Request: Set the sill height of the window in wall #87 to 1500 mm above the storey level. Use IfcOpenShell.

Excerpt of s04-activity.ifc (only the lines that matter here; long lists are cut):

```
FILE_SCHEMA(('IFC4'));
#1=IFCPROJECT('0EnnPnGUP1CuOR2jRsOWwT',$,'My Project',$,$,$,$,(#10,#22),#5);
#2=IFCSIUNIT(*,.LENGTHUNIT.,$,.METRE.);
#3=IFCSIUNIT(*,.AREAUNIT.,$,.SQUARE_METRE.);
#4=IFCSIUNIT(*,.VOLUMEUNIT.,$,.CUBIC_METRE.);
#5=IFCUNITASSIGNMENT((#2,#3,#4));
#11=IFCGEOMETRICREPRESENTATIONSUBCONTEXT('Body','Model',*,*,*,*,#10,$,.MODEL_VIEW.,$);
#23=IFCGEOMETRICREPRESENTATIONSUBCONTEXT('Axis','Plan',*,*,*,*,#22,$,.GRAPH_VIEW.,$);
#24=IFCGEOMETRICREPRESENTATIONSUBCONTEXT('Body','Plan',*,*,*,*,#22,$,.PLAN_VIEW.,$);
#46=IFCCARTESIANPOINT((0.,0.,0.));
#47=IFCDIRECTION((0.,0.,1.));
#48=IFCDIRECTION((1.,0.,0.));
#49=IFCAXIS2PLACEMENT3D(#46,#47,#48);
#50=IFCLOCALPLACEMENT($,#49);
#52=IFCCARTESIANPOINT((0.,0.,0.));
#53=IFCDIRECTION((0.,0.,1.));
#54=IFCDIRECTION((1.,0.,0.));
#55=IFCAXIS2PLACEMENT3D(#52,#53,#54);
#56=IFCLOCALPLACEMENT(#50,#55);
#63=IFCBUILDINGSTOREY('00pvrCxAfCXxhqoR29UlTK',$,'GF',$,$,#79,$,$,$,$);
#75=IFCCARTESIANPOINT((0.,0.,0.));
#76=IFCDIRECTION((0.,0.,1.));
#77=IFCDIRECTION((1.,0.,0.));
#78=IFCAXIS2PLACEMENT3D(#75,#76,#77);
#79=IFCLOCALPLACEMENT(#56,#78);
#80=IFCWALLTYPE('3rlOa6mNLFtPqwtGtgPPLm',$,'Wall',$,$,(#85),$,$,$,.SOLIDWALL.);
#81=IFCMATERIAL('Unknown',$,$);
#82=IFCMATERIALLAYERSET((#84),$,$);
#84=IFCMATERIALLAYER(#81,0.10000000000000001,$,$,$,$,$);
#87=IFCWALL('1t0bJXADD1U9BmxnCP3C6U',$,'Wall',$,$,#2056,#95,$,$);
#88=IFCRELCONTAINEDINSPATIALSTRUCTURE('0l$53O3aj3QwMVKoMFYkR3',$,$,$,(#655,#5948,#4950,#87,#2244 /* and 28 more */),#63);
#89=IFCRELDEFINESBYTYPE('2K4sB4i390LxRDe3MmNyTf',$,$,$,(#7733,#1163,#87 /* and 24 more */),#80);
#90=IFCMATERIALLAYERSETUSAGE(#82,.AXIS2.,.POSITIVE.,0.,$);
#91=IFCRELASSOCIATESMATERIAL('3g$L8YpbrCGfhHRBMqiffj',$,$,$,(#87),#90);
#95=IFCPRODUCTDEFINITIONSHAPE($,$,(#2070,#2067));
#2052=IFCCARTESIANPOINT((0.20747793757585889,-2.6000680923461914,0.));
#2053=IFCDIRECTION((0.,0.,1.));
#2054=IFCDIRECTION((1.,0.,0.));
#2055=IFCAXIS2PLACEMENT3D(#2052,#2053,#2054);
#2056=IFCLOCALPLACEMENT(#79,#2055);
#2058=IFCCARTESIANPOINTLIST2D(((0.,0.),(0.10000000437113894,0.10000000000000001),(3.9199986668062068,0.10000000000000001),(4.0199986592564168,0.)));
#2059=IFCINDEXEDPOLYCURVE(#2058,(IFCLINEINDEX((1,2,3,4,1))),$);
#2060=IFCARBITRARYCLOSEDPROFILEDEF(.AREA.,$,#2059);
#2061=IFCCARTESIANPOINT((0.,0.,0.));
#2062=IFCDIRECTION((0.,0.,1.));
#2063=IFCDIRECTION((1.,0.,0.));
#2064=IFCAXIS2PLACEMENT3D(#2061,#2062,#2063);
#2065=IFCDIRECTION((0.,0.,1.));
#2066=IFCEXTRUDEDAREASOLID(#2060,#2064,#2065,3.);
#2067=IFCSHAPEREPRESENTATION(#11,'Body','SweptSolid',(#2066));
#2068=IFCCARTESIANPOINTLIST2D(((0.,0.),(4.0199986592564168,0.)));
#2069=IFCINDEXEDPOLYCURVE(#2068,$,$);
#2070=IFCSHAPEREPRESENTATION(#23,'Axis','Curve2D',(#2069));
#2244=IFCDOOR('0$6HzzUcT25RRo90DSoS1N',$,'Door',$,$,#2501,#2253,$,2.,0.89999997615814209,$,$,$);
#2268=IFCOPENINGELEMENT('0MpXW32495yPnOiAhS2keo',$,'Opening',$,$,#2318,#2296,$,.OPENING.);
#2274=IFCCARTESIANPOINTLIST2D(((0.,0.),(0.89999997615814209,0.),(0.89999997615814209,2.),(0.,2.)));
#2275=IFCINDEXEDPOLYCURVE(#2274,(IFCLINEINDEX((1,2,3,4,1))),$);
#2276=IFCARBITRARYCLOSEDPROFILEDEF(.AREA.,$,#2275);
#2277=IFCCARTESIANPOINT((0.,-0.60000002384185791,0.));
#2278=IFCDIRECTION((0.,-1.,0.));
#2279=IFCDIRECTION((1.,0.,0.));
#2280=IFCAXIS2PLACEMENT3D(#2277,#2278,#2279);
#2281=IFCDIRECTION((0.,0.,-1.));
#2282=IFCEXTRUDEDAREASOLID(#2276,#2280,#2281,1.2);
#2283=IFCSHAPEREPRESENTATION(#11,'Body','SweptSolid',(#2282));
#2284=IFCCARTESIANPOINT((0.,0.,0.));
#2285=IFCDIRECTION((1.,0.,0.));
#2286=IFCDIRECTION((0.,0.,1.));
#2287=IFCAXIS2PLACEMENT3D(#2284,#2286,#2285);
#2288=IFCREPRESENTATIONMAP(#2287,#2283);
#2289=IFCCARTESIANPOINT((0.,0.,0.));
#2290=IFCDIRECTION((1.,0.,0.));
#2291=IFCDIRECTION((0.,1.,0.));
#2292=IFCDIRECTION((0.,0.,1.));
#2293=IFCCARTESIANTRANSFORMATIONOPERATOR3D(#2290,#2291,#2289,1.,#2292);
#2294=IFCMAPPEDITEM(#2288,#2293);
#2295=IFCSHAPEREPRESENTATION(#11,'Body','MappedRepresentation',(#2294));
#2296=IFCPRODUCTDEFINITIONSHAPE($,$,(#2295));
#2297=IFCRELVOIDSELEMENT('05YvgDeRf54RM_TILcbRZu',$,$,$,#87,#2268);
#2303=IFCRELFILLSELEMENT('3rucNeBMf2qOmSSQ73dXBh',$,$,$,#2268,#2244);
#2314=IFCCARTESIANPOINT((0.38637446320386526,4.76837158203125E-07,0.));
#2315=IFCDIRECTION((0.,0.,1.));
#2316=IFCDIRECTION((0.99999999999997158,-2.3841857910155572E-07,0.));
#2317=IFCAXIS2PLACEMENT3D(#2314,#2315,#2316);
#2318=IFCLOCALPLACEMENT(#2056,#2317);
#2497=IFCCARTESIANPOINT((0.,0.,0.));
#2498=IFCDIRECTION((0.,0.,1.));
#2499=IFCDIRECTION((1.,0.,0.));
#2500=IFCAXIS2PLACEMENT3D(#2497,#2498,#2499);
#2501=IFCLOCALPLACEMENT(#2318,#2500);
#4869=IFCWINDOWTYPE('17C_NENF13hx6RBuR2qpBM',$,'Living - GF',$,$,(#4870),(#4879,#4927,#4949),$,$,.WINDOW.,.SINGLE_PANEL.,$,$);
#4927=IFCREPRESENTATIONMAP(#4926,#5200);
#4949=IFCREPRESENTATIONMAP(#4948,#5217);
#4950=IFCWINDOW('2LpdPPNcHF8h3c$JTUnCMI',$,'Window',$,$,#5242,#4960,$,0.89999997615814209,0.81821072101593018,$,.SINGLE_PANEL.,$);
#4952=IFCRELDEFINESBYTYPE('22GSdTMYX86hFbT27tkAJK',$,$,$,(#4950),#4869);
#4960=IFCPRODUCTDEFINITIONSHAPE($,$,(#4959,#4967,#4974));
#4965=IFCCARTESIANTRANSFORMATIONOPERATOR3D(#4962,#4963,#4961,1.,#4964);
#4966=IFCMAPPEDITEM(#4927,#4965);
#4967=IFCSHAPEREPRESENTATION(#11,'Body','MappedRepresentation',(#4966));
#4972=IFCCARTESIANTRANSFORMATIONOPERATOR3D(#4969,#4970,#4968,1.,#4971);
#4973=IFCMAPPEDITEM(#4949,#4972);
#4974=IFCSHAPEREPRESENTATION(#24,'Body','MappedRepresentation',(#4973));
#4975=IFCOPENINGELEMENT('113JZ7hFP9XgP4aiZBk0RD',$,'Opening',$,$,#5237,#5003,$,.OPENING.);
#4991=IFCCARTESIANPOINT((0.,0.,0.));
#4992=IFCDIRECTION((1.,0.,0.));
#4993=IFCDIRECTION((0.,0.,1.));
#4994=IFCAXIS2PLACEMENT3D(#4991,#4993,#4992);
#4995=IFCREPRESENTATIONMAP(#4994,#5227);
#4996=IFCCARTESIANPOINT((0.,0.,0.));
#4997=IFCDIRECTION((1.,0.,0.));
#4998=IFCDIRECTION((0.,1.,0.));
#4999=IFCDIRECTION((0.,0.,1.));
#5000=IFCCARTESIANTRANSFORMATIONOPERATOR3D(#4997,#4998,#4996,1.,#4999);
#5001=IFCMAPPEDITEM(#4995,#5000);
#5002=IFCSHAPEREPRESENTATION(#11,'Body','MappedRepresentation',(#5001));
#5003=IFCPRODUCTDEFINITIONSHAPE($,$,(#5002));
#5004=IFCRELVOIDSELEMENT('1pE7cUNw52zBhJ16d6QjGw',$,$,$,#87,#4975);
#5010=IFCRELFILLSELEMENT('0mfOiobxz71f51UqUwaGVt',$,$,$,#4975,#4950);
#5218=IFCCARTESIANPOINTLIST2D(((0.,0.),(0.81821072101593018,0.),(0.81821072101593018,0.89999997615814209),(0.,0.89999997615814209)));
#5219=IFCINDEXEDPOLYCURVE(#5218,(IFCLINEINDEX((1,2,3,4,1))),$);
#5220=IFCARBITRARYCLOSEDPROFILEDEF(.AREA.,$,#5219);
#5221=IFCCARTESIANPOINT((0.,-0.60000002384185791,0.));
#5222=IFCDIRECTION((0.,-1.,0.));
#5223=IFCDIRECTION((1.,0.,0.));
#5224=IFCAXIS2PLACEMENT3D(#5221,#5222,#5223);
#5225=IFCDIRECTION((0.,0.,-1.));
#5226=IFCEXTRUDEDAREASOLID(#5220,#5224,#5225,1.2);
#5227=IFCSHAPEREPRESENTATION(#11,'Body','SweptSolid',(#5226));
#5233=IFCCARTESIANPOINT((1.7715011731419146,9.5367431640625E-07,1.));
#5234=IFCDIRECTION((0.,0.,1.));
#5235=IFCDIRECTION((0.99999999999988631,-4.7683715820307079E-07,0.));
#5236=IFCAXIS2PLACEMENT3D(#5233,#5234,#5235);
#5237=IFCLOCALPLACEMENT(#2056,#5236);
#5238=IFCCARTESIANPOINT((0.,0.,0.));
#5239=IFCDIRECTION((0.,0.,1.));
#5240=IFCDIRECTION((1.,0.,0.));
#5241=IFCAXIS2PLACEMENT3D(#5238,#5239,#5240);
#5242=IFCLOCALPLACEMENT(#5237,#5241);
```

```python
import numpy as np
import ifcopenshell
import ifcopenshell.api.geometry
import ifcopenshell.geom
import ifcopenshell.util.element
import ifcopenshell.util.placement
import ifcopenshell.util.shape
import ifcopenshell.util.unit

model = ifcopenshell.open("s04-activity.ifc")
unit_scale = ifcopenshell.util.unit.calculate_unit_scale(model)

window = model.by_guid("2LpdPPNcHF8h3c$JTUnCMI")
opening = window.FillsVoids[0].RelatingOpeningElement
storey = ifcopenshell.util.element.get_container(window, ifc_class="IfcBuildingStorey")
level = ifcopenshell.util.placement.get_local_placement(storey.ObjectPlacement)[2, 3]

# The opening's origin need not be at the sill, so measure its lowest point.
shape = ifcopenshell.geom.create_shape(ifcopenshell.geom.settings(), opening)
bottom = ifcopenshell.util.shape.get_shape_bottom_elevation(shape, shape.geometry) / unit_scale
dz = level + 1.5 / unit_scale - bottom

shift = np.array([0.0, 0.0, dz])
# The window is placed relative to its opening, so it follows when the opening moves.
matrix = ifcopenshell.util.placement.get_local_placement(opening.ObjectPlacement)
matrix[:3, 3] += shift
ifcopenshell.api.geometry.edit_object_placement(
    model, product=opening, matrix=matrix, is_si=False, should_transform_children=True
)

print(f"moved by {dz * unit_scale:+.3f} m")

model.write("s04-activity_edited.ifc")
```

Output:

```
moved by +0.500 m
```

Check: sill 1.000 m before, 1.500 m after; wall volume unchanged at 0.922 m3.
